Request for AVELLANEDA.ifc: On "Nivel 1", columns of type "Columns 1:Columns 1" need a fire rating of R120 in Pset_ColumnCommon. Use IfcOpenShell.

First a look at what the model holds.

```python
import ifcopenshell
import ifcopenshell.util.element

model = ifcopenshell.open("AVELLANEDA.ifc")
print(model.schema)
storey = next(s for s in model.by_type("IfcBuildingStorey") if s.Name == "Nivel 1")
columns = [e for e in ifcopenshell.util.element.get_decomposition(storey) if e.is_a("IfcColumn")]
seen = {}
for e in columns:
    element_type = ifcopenshell.util.element.get_type(e)
    key = (element_type.Name if element_type != e and element_type else None, ifcopenshell.util.element.get_pset(e, "Pset_ColumnCommon", "FireRating"))
    seen[key] = seen.get(key, 0) + 1
for (name, value), count in sorted(seen.items(), key=str):
    print(count, "x", name, "|", value)
```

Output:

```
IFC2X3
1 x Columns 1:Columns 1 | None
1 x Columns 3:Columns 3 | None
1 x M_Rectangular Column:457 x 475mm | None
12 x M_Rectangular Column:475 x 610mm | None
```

```python
import ifcopenshell
import ifcopenshell.api.pset
import ifcopenshell.util.element

model = ifcopenshell.open("AVELLANEDA.ifc")

storey = next(s for s in model.by_type("IfcBuildingStorey") if s.Name == "Nivel 1")
columns = [e for e in ifcopenshell.util.element.get_decomposition(storey) if e.is_a("IfcColumn")]

count = 0
for e in columns:
    element_type = ifcopenshell.util.element.get_type(e)
    if element_type in (None, e) or element_type.Name != "Columns 1:Columns 1":
        continue
    # add_pset returns the element's existing set when there is one.
    pset = ifcopenshell.api.pset.add_pset(model, product=e, name="Pset_ColumnCommon")
    ifcopenshell.api.pset.edit_pset(model, pset=pset, properties={"FireRating": "R120"})
    count += 1

print(count, "columns updated")

model.write("AVELLANEDA-out.ifc")
```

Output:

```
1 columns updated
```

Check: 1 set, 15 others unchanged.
